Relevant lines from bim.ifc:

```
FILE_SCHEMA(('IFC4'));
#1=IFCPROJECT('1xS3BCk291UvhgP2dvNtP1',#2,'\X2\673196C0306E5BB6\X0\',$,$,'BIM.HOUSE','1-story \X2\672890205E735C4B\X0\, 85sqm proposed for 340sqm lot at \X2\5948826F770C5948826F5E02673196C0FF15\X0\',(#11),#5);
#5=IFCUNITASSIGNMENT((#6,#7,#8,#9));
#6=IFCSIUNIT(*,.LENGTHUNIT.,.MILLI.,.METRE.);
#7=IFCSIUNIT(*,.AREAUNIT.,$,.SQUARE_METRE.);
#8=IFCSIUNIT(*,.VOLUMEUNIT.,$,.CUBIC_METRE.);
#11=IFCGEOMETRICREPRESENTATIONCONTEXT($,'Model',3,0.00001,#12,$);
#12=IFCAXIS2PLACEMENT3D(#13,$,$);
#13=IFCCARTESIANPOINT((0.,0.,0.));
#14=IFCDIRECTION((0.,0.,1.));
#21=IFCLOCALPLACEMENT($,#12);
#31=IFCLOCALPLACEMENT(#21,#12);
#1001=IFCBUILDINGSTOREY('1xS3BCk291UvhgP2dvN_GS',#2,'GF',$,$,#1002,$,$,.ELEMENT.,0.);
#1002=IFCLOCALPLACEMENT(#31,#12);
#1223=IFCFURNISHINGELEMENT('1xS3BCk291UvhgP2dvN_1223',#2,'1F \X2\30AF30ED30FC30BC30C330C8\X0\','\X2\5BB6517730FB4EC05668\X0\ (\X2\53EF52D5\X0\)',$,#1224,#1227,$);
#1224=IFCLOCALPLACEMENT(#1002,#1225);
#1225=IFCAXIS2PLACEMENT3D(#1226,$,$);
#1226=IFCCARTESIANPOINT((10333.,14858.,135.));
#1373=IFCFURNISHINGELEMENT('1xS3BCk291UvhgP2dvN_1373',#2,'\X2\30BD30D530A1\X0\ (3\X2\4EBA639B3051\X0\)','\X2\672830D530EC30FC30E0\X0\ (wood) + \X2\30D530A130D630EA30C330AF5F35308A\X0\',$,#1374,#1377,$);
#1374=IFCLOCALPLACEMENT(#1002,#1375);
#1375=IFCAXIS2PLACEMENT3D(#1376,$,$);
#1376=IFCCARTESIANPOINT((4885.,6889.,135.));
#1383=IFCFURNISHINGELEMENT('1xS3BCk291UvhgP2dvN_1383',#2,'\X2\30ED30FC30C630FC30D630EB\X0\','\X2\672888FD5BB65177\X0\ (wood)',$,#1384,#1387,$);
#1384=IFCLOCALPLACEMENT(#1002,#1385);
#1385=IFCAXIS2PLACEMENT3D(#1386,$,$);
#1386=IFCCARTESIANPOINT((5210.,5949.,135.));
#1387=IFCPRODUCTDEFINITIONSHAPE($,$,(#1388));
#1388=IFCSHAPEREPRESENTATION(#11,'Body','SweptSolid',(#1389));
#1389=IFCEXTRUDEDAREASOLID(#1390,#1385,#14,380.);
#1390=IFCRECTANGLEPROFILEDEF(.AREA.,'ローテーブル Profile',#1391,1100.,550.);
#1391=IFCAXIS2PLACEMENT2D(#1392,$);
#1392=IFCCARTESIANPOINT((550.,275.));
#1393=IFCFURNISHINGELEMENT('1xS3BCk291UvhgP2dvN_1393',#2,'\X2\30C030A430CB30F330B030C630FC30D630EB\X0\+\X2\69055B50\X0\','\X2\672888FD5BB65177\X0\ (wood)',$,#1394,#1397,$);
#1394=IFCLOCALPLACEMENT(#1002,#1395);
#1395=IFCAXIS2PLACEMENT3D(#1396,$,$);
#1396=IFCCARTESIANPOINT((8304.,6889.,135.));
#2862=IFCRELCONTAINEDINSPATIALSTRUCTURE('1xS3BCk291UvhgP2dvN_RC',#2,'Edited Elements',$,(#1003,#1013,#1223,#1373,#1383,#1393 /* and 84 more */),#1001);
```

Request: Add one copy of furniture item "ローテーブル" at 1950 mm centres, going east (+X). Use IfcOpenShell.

```python
import numpy as np
import ifcopenshell
import ifcopenshell.api.geometry
import ifcopenshell.api.root
import ifcopenshell.util.element
import ifcopenshell.util.placement
import ifcopenshell.util.unit

model = ifcopenshell.open("bim.ifc")
unit_scale = ifcopenshell.util.unit.calculate_unit_scale(model)


def reuse_history(source, copy):
    """copy_class also copies each property set's owner history, people and application; keep the originals."""
    for rel in copy.IsDefinedBy:
        if rel.is_a("IfcRelDefinesByProperties") and (history := rel.RelatingPropertyDefinition.OwnerHistory):
            rel.RelatingPropertyDefinition.OwnerHistory = source.OwnerHistory
            ifcopenshell.util.element.remove_deep2(model, history)


source = model.by_id(1383)
base = ifcopenshell.util.placement.get_local_placement(source.ObjectPlacement)
step = np.array([1.0, 0.0, 0.0]) * 1.95 / unit_scale

for i in range(1, 2):
    copy = ifcopenshell.api.root.copy_class(model, product=source)
    copy.Representation = ifcopenshell.util.element.copy_deep(
        model, source.Representation, exclude=["IfcGeometricRepresentationContext", "IfcRepresentationMap"]
    )
    reuse_history(source, copy)
    matrix = base.copy()
    matrix[:3, 3] += i * step
    print("added at", matrix[:3, 3].round(3) + 0.0)
    ifcopenshell.api.geometry.edit_object_placement(model, product=copy, matrix=matrix, is_si=False)

model.write("bim_edited.ifc")
```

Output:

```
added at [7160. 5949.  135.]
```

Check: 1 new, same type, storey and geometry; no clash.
